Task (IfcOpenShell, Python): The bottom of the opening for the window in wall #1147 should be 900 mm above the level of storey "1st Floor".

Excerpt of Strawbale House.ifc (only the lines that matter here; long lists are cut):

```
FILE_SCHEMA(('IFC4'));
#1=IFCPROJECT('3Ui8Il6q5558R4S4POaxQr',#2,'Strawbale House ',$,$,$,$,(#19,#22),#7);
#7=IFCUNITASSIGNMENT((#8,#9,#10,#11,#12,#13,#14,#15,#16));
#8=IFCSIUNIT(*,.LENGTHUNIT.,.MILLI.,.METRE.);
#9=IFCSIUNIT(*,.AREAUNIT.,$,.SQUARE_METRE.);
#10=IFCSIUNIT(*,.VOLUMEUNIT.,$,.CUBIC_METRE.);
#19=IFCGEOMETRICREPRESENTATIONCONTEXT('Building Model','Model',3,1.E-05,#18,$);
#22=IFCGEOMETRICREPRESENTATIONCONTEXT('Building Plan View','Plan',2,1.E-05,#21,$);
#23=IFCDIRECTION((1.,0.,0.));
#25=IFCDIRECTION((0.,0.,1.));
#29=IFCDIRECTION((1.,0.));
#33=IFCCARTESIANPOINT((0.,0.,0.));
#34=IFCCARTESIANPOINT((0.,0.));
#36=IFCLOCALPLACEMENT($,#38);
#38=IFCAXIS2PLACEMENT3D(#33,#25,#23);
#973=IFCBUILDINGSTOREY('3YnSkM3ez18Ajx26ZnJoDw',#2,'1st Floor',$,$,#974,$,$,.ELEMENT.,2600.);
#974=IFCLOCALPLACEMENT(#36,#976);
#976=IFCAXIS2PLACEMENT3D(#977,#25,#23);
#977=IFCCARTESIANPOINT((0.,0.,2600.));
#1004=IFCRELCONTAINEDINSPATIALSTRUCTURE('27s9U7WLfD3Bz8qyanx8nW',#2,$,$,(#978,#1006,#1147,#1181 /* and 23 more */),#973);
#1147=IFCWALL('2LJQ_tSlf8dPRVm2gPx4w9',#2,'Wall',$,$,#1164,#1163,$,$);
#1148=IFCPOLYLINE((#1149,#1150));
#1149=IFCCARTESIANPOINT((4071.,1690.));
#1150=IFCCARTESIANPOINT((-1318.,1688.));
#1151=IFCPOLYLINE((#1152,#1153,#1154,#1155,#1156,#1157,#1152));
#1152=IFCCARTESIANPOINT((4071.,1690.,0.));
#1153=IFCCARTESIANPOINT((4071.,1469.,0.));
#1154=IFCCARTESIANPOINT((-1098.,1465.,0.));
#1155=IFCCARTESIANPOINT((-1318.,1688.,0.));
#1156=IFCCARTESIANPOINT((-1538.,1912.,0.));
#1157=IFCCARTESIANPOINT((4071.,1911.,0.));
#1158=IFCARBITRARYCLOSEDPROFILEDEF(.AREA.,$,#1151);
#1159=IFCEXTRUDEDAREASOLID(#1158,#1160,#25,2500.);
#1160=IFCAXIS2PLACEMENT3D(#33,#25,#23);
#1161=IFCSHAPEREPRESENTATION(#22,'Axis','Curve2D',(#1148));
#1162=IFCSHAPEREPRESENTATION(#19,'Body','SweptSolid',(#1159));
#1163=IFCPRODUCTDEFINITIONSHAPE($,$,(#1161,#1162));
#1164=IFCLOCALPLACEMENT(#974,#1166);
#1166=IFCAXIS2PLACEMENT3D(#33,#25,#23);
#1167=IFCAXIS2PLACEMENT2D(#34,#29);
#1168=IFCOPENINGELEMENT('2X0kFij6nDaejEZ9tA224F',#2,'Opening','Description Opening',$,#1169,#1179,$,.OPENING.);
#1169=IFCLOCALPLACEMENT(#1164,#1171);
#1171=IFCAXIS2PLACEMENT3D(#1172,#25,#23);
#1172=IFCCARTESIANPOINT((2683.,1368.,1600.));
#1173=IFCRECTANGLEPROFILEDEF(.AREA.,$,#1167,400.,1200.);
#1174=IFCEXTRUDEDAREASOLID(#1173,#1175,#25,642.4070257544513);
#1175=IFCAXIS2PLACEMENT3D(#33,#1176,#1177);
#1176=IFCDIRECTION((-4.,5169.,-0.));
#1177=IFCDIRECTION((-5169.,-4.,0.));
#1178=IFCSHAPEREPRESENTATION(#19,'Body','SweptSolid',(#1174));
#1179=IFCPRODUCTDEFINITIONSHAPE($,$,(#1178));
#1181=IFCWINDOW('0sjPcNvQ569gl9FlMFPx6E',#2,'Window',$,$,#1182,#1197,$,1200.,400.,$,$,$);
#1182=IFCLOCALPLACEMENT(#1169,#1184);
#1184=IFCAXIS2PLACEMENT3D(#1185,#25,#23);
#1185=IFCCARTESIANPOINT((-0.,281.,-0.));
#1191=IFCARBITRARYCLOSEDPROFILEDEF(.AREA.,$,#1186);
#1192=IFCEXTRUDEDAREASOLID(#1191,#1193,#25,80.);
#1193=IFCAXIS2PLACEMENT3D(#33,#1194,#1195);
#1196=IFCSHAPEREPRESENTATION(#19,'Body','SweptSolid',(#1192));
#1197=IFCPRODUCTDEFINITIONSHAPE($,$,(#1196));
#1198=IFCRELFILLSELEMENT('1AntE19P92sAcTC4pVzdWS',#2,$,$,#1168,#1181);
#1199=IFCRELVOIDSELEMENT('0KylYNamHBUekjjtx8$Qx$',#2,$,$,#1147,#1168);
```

```python
import numpy as np
import ifcopenshell
import ifcopenshell.api.geometry
import ifcopenshell.geom
import ifcopenshell.util.element
import ifcopenshell.util.placement
import ifcopenshell.util.shape
import ifcopenshell.util.unit

model = ifcopenshell.open("Strawbale House.ifc")
unit_scale = ifcopenshell.util.unit.calculate_unit_scale(model)

window = model.by_guid("0sjPcNvQ569gl9FlMFPx6E")
opening = window.FillsVoids[0].RelatingOpeningElement
storey = ifcopenshell.util.element.get_container(window, ifc_class="IfcBuildingStorey")
level = ifcopenshell.util.placement.get_local_placement(storey.ObjectPlacement)[2, 3]

# The opening's origin need not be at the sill, so measure its lowest point.
shape = ifcopenshell.geom.create_shape(ifcopenshell.geom.settings(), opening)
bottom = ifcopenshell.util.shape.get_shape_bottom_elevation(shape, shape.geometry) / unit_scale
dz = level + 0.9 / unit_scale - bottom

shift = np.array([0.0, 0.0, dz])
# The window is placed relative to its opening, so it follows when the opening moves.
matrix = ifcopenshell.util.placement.get_local_placement(opening.ObjectPlacement)
matrix[:3, 3] += shift
ifcopenshell.api.geometry.edit_object_placement(
    model, product=opening, matrix=matrix, is_si=False, should_transform_children=True
)

print(f"moved by {dz * unit_scale:+.3f} m")

model.write("Strawbale House_updated.ifc")
```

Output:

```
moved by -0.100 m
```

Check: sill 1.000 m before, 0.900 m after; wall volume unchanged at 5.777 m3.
